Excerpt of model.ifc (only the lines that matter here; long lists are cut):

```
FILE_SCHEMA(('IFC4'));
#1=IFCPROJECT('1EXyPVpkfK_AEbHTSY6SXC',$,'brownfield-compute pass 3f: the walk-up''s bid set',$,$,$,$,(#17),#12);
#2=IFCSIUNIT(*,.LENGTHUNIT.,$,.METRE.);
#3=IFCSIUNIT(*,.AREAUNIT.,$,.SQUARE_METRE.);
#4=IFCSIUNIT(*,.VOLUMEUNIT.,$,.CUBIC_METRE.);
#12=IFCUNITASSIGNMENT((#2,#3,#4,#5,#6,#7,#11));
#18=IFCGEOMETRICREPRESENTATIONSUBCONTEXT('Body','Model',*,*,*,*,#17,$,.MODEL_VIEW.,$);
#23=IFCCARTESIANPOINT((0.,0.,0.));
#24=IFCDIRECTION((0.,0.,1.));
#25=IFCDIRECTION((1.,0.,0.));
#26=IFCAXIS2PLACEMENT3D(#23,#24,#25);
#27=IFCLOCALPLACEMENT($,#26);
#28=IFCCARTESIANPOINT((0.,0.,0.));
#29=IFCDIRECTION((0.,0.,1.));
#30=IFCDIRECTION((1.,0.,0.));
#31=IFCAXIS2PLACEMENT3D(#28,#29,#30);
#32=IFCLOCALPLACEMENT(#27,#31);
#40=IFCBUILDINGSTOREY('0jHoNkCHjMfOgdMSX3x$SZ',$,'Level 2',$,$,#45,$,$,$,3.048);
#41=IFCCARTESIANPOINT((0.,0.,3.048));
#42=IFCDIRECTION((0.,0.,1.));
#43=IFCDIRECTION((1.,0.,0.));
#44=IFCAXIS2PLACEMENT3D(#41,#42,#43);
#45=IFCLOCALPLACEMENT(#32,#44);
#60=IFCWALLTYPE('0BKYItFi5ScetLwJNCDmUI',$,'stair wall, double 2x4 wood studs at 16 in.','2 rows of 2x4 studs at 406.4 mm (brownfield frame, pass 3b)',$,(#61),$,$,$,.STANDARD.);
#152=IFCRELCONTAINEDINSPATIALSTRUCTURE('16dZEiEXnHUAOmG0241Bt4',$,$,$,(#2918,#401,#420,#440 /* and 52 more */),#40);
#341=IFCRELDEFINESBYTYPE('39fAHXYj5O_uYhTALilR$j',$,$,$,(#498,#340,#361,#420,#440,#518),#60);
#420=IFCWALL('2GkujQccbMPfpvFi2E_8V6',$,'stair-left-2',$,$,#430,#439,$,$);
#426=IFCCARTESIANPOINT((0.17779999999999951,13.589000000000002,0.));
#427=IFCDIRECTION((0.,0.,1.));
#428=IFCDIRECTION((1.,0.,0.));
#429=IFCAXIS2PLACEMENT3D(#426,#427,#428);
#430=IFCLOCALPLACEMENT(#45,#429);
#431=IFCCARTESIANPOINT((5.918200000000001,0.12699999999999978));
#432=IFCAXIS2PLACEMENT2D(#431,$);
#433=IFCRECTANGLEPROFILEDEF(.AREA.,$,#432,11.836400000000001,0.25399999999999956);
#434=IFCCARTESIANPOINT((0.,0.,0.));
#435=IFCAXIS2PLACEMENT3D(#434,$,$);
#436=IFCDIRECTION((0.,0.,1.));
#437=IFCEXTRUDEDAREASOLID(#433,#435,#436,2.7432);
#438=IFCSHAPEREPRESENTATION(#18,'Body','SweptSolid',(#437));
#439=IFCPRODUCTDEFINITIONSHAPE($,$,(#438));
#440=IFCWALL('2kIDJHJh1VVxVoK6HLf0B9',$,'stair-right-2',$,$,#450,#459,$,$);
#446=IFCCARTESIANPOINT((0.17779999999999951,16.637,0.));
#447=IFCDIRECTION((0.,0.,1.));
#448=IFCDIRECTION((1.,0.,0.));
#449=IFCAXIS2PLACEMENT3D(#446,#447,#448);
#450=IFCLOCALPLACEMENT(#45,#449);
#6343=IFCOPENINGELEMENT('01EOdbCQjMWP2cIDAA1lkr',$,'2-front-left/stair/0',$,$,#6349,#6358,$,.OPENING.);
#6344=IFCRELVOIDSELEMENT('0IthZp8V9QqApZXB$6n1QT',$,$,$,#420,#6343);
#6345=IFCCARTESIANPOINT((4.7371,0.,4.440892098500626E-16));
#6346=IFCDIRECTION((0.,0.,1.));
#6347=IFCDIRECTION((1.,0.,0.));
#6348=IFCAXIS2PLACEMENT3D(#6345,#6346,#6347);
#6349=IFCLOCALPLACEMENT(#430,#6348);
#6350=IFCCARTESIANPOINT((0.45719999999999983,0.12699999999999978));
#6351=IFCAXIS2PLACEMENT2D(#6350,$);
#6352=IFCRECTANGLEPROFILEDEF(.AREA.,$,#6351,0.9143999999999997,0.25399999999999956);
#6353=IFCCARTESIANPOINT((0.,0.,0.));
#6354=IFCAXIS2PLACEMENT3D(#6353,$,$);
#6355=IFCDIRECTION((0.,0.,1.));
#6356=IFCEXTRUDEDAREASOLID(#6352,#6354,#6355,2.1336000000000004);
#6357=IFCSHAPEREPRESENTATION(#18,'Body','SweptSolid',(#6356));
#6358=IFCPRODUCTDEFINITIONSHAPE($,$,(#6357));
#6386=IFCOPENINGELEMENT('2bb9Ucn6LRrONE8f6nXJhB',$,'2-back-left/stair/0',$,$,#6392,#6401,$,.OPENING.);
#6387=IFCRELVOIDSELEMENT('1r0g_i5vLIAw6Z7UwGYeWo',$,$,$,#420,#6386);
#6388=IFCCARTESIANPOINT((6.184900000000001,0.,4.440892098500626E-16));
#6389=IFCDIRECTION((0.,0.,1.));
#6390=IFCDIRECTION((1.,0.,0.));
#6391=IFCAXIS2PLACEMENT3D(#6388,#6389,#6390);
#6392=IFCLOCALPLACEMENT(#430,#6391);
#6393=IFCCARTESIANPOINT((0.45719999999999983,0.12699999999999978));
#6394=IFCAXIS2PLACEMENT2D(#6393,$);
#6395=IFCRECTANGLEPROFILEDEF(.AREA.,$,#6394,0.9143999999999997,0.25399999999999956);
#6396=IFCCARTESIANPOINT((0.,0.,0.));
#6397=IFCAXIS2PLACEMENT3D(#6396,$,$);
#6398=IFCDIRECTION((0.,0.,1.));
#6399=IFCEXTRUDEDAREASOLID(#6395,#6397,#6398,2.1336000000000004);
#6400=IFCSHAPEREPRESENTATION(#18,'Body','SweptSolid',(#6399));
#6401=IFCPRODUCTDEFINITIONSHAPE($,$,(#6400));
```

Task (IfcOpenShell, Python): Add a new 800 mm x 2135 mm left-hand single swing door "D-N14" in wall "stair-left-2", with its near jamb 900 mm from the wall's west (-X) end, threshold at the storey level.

```python
import numpy as np
import ifcopenshell
import ifcopenshell.api.feature
import ifcopenshell.api.geometry
import ifcopenshell.api.root
import ifcopenshell.api.spatial
import ifcopenshell.geom
import ifcopenshell.util.element
import ifcopenshell.util.placement
import ifcopenshell.util.representation
import ifcopenshell.util.shape
import ifcopenshell.util.unit

model = ifcopenshell.open("model.ifc")
unit_scale = ifcopenshell.util.unit.calculate_unit_scale(model)
settings = ifcopenshell.geom.settings()


def volume(element):
    """Net volume in cubic metres, openings subtracted."""
    shape = ifcopenshell.geom.create_shape(settings, element)
    return ifcopenshell.util.shape.get_volume(shape.geometry)


wall = model.by_guid("2GkujQccbMPfpvFi2E_8V6")
storey = ifcopenshell.util.element.get_container(wall, ifc_class="IfcBuildingStorey")
context = ifcopenshell.util.representation.get_context(model, "Model", "Body", "MODEL_VIEW")
before = volume(wall)

width, height, from_end, sill = 0.8, 2.135, 0.9, 0.0  # metres

# The wall runs along its own X axis, and the end named is its -X end.
wall_shape = ifcopenshell.geom.create_shape(settings, wall)
x, y, z = ifcopenshell.util.shape.get_vertices(wall_shape.geometry).T
start = x.min() + from_end
face, thickness = float(y.min()), float(y.max() - y.min())
wall_matrix = ifcopenshell.util.placement.get_local_placement(wall.ObjectPlacement)
level = ifcopenshell.util.placement.get_local_placement(storey.ObjectPlacement)[2, 3]


def in_wall(x, y):
    """Placement at x, y metres in the wall's axes, at sill height."""
    matrix = wall_matrix.copy()
    matrix[:, 3] = wall_matrix @ np.array([x / unit_scale, y / unit_scale, 0.0, 1.0])
    matrix[2, 3] = level + sill / unit_scale
    return matrix


# Opening: a box that overshoots both wall faces by 50 mm.
opening = ifcopenshell.api.root.create_entity(model, ifc_class="IfcOpeningElement", predefined_type="OPENING")
box = ifcopenshell.api.geometry.add_wall_representation(
    model, context=context, length=width, height=height, thickness=thickness + 0.1
)
ifcopenshell.api.geometry.assign_representation(model, product=opening, representation=box)
ifcopenshell.api.geometry.edit_object_placement(model, product=opening, matrix=in_wall(start, face - 0.05), is_si=False)
ifcopenshell.api.feature.add_feature(model, feature=opening, element=wall)

door = ifcopenshell.api.root.create_entity(model, ifc_class="IfcDoor", name="D-N14", predefined_type="DOOR")
door.OverallWidth, door.OverallHeight = width / unit_scale, height / unit_scale
door.OperationType = "SINGLE_SWING_LEFT"
body = ifcopenshell.api.geometry.add_door_representation(
    model,
    context=context,
    overall_width=door.OverallWidth,
    overall_height=door.OverallHeight,
    operation_type="SINGLE_SWING_LEFT",
    lining_properties={"LiningDepth": thickness / unit_scale, "ThresholdDepth": thickness / unit_scale},
)
ifcopenshell.api.geometry.assign_representation(model, product=door, representation=body)
ifcopenshell.api.spatial.assign_container(model, products=[door], relating_structure=storey)
ifcopenshell.api.feature.add_filling(model, opening=opening, element=door)

# The lining spans the wall, so the door starts at the wall face.
ifcopenshell.api.geometry.edit_object_placement(model, product=door, matrix=in_wall(start, face), is_si=False)

after = volume(wall)

print(f"wall volume {before:.3f} -> {after:.3f} m3")

model.write("model_rev.ifc")
```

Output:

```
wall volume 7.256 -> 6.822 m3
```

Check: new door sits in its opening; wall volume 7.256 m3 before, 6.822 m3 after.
